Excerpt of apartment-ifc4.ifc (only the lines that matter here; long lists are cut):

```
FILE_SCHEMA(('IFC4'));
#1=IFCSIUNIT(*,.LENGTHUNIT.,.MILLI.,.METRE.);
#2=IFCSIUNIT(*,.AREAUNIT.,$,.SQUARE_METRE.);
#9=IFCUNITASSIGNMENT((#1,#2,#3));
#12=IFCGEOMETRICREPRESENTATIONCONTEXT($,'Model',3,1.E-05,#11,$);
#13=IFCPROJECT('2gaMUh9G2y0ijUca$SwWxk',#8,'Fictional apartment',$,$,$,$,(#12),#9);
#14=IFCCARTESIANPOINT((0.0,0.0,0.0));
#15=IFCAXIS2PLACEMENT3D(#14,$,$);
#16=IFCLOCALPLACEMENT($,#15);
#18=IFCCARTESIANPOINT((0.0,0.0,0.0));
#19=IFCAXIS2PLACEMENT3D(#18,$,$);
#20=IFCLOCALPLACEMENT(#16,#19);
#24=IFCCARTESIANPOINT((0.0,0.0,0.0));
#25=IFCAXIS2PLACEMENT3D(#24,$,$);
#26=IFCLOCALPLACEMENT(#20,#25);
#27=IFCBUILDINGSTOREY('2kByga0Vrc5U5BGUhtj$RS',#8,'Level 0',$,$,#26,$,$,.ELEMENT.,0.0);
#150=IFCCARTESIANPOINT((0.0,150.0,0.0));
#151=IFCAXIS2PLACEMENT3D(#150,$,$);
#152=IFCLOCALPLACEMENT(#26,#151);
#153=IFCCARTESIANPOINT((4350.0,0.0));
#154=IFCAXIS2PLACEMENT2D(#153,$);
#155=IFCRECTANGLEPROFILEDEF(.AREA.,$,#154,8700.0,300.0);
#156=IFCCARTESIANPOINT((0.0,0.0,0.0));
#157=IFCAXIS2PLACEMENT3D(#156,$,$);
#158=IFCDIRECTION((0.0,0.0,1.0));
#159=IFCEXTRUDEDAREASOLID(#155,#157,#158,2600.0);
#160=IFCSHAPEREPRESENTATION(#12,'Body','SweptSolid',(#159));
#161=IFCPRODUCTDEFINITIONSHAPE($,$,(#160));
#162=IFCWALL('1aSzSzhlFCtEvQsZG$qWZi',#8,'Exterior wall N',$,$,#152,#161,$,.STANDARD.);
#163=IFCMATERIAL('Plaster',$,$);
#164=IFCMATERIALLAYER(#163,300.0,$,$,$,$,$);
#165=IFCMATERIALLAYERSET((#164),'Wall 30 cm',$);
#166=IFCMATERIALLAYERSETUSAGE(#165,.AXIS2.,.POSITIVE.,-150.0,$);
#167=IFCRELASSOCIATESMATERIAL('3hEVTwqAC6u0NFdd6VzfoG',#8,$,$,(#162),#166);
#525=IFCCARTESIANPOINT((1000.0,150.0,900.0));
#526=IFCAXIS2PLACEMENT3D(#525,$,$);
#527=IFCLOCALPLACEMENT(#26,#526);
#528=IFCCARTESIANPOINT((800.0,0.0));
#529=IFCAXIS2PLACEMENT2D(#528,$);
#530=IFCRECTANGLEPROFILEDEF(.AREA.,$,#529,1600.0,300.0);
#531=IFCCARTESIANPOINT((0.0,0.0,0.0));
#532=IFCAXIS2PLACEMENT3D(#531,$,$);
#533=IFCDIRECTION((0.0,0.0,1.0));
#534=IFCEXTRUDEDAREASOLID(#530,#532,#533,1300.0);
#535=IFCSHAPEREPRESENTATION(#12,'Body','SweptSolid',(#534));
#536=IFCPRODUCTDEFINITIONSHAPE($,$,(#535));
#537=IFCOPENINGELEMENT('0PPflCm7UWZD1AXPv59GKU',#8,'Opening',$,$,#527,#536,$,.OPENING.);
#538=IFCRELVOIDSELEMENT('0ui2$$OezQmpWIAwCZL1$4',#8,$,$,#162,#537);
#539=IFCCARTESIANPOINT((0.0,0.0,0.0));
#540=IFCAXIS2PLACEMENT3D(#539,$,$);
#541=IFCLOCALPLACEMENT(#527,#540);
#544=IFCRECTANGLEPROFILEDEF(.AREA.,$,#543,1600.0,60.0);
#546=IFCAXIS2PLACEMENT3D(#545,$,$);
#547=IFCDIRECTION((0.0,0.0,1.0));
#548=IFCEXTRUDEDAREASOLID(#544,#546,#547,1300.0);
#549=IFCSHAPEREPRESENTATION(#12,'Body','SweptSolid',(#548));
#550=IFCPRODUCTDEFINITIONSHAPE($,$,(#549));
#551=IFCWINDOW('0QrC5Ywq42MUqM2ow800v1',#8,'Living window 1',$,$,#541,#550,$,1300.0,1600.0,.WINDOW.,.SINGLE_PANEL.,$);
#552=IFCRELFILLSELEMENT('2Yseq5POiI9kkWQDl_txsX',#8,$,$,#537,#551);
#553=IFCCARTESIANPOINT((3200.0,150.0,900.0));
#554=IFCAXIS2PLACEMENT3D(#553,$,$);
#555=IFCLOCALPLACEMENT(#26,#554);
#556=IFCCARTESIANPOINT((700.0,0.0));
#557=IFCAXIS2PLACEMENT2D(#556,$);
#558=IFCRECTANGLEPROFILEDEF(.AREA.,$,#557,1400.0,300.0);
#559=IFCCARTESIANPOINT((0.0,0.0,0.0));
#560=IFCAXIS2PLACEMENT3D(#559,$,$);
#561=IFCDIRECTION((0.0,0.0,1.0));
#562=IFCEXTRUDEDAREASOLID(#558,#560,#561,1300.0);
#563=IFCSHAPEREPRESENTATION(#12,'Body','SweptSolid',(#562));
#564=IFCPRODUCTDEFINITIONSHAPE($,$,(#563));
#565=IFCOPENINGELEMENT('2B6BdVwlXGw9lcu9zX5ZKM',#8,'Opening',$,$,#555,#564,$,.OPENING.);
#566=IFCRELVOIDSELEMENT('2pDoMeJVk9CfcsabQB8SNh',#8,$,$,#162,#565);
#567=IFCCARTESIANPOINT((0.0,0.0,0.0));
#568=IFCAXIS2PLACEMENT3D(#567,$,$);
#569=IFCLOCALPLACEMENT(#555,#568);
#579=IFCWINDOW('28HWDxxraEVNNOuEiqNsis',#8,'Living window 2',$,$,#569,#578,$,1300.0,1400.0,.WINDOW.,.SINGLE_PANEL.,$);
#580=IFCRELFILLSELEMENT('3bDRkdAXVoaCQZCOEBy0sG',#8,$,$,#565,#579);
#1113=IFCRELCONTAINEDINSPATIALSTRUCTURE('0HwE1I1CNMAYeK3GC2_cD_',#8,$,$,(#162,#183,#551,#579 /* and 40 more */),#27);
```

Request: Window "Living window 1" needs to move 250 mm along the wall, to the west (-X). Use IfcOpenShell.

```python
import ifcopenshell
import ifcopenshell.api.geometry
import ifcopenshell.util.placement
import ifcopenshell.util.unit

model = ifcopenshell.open("apartment-ifc4.ifc")
unit_scale = ifcopenshell.util.unit.calculate_unit_scale(model)

window = model.by_id(551)
opening = window.FillsVoids[0].RelatingOpeningElement
wall = opening.VoidsElements[0].RelatingBuildingElement

wall_matrix = ifcopenshell.util.placement.get_local_placement(wall.ObjectPlacement)
shift = wall_matrix[:3, 0] * -0.25 / unit_scale
before = ifcopenshell.util.placement.get_local_placement(window.ObjectPlacement)[:3, 3].copy()

# The window is placed relative to its opening, so it follows when the opening moves.
matrix = ifcopenshell.util.placement.get_local_placement(opening.ObjectPlacement)
matrix[:3, 3] += shift
ifcopenshell.api.geometry.edit_object_placement(
    model, product=opening, matrix=matrix, is_si=False, should_transform_children=True
)

after = ifcopenshell.util.placement.get_local_placement(window.ObjectPlacement)[:3, 3]
print("window moved by", (after - before).round(3) + 0.0)

model.write("apartment-ifc4-out.ifc")
```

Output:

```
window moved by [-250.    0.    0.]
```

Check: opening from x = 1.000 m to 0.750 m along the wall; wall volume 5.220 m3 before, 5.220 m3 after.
